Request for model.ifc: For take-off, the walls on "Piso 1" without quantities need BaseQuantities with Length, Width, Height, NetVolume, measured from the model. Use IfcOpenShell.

First a look at what the model holds.

```python
import ifcopenshell
import ifcopenshell.util.element
import ifcopenshell.util.unit

model = ifcopenshell.open("model.ifc")
print(model.schema)
for unit_type in ("LENGTHUNIT", "AREAUNIT", "VOLUMEUNIT"):
    print(unit_type, ifcopenshell.util.unit.calculate_unit_scale(model, unit_type))
storey = next(s for s in model.by_type("IfcBuildingStorey") if s.Name == "Piso 1")
walls = [e for e in ifcopenshell.util.element.get_decomposition(storey) if e.is_a("IfcWall")]
for e in sorted(walls, key=lambda e: e.id()):
    print(e.id(), e.is_a(), e.Name, list(ifcopenshell.util.element.get_psets(e, qtos_only=True)), sep=" | ")
```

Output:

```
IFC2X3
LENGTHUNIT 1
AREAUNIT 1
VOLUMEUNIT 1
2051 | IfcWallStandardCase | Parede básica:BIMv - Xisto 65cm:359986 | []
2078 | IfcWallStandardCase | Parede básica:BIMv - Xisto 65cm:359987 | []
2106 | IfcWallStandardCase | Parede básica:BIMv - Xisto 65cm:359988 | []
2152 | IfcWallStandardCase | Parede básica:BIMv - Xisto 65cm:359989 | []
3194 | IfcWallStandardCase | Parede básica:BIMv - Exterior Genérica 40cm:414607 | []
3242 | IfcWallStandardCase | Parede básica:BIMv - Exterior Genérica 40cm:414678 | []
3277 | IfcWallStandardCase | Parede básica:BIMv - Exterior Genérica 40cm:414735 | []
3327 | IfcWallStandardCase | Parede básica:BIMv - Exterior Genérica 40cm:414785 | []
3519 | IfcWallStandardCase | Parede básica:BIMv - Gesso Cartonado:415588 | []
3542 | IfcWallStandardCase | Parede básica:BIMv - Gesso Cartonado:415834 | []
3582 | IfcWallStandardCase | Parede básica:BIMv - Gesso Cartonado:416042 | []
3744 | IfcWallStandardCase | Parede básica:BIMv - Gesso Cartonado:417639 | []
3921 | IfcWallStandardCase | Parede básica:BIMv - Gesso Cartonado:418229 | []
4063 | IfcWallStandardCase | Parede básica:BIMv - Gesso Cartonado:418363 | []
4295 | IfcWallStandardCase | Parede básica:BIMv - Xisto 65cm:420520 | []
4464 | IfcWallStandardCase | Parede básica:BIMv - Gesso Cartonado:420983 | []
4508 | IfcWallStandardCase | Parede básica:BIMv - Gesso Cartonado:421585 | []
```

```python
import ifcopenshell
import ifcopenshell.api.pset
import ifcopenshell.geom
import ifcopenshell.util.element
import ifcopenshell.util.shape
import ifcopenshell.util.unit

model = ifcopenshell.open("model.ifc")
unit_scale = ifcopenshell.util.unit.calculate_unit_scale(model)
volume_scale = ifcopenshell.util.unit.calculate_unit_scale(model, "VOLUMEUNIT")
settings = ifcopenshell.geom.settings()

storey = next(s for s in model.by_type("IfcBuildingStorey") if s.Name == "Piso 1")
walls = [e for e in ifcopenshell.util.element.get_decomposition(storey) if e.is_a("IfcWall")]

for e in sorted(walls, key=lambda e: e.id()):
    if ifcopenshell.util.element.get_psets(e, qtos_only=True, should_inherit=False):
        continue
    # Geometry comes back in metres, in the element's own axes.
    shape = ifcopenshell.geom.create_shape(settings, e)
    values = {
        "Length": ifcopenshell.util.shape.get_x(shape.geometry) / unit_scale,
        "Width": ifcopenshell.util.shape.get_y(shape.geometry) / unit_scale,
        "Height": ifcopenshell.util.shape.get_z(shape.geometry) / unit_scale,
        "NetVolume": ifcopenshell.util.shape.get_volume(shape.geometry) / volume_scale,
    }
    qto = ifcopenshell.api.pset.add_qto(model, product=e, name="BaseQuantities")
    ifcopenshell.api.pset.edit_qto(model, qto=qto, properties=values)
    print(e.id(), {k: round(v, 3) for k, v in values.items()})

model.write("model-out.ifc")
```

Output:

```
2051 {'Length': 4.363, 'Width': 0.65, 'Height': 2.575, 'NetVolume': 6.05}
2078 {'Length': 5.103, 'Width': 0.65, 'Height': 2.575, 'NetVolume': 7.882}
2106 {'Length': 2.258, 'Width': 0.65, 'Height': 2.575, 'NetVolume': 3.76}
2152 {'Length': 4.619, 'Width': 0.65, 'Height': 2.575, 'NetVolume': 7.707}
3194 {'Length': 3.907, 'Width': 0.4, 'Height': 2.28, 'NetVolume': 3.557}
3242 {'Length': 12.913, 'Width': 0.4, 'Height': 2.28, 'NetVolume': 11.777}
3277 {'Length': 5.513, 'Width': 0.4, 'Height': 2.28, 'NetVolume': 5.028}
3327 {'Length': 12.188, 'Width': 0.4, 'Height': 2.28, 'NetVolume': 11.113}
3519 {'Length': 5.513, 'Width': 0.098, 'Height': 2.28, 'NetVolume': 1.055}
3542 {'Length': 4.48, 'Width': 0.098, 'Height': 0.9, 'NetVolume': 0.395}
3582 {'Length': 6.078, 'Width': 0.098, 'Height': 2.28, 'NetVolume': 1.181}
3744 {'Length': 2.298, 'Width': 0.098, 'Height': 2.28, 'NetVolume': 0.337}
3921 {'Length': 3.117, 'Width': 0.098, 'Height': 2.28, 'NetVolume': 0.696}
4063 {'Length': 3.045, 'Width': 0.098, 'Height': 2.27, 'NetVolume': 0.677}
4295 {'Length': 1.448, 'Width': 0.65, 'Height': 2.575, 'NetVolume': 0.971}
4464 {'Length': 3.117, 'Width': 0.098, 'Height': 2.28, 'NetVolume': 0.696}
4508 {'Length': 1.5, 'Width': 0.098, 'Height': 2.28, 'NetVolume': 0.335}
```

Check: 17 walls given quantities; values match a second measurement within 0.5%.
